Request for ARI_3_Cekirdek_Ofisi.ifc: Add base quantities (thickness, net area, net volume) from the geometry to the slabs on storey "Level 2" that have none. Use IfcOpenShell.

First a look at what the model holds.

```python
import ifcopenshell
import ifcopenshell.util.element
import ifcopenshell.util.unit

model = ifcopenshell.open("ARI_3_Cekirdek_Ofisi.ifc")
print(model.schema)
for unit_type in ("LENGTHUNIT", "AREAUNIT", "VOLUMEUNIT"):
    print(unit_type, ifcopenshell.util.unit.calculate_unit_scale(model, unit_type))
storey = next(s for s in model.by_type("IfcBuildingStorey") if s.Name == "Level 2")
slabs = [e for e in ifcopenshell.util.element.get_decomposition(storey) if e.is_a("IfcSlab")]
for e in sorted(slabs, key=lambda e: e.id()):
    print(e.id(), e.is_a(), e.Name, list(ifcopenshell.util.element.get_psets(e, qtos_only=True)), sep=" | ")
```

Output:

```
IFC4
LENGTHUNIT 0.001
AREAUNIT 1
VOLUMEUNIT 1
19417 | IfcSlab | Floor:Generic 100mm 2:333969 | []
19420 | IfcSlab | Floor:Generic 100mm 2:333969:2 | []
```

```python
import ifcopenshell
import ifcopenshell.api.pset
import ifcopenshell.geom
import ifcopenshell.util.element
import ifcopenshell.util.shape
import ifcopenshell.util.unit

model = ifcopenshell.open("ARI_3_Cekirdek_Ofisi.ifc")
unit_scale = ifcopenshell.util.unit.calculate_unit_scale(model)
area_scale = ifcopenshell.util.unit.calculate_unit_scale(model, "AREAUNIT")
volume_scale = ifcopenshell.util.unit.calculate_unit_scale(model, "VOLUMEUNIT")
settings = ifcopenshell.geom.settings()

storey = next(s for s in model.by_type("IfcBuildingStorey") if s.Name == "Level 2")
slabs = [e for e in ifcopenshell.util.element.get_decomposition(storey) if e.is_a("IfcSlab")]

for e in sorted(slabs, key=lambda e: e.id()):
    if ifcopenshell.util.element.get_psets(e, qtos_only=True, should_inherit=False):
        continue
    # Geometry comes back in metres, in the element's own axes.
    shape = ifcopenshell.geom.create_shape(settings, e)
    values = {
        "Width": ifcopenshell.util.shape.get_z(shape.geometry) / unit_scale,
        "NetArea": ifcopenshell.util.shape.get_footprint_area(shape.geometry) / area_scale,
        "NetVolume": ifcopenshell.util.shape.get_volume(shape.geometry) / volume_scale,
    }
    qto = ifcopenshell.api.pset.add_qto(model, product=e, name="Qto_SlabBaseQuantities")
    ifcopenshell.api.pset.edit_qto(model, qto=qto, properties=values)
    print(e.id(), {k: round(v, 3) for k, v in values.items()})

model.write("ARI_3_Cekirdek_Ofisi_v2.ifc")
```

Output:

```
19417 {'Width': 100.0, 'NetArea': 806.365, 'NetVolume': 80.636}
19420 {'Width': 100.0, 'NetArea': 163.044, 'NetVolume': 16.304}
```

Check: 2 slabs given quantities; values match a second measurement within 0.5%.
